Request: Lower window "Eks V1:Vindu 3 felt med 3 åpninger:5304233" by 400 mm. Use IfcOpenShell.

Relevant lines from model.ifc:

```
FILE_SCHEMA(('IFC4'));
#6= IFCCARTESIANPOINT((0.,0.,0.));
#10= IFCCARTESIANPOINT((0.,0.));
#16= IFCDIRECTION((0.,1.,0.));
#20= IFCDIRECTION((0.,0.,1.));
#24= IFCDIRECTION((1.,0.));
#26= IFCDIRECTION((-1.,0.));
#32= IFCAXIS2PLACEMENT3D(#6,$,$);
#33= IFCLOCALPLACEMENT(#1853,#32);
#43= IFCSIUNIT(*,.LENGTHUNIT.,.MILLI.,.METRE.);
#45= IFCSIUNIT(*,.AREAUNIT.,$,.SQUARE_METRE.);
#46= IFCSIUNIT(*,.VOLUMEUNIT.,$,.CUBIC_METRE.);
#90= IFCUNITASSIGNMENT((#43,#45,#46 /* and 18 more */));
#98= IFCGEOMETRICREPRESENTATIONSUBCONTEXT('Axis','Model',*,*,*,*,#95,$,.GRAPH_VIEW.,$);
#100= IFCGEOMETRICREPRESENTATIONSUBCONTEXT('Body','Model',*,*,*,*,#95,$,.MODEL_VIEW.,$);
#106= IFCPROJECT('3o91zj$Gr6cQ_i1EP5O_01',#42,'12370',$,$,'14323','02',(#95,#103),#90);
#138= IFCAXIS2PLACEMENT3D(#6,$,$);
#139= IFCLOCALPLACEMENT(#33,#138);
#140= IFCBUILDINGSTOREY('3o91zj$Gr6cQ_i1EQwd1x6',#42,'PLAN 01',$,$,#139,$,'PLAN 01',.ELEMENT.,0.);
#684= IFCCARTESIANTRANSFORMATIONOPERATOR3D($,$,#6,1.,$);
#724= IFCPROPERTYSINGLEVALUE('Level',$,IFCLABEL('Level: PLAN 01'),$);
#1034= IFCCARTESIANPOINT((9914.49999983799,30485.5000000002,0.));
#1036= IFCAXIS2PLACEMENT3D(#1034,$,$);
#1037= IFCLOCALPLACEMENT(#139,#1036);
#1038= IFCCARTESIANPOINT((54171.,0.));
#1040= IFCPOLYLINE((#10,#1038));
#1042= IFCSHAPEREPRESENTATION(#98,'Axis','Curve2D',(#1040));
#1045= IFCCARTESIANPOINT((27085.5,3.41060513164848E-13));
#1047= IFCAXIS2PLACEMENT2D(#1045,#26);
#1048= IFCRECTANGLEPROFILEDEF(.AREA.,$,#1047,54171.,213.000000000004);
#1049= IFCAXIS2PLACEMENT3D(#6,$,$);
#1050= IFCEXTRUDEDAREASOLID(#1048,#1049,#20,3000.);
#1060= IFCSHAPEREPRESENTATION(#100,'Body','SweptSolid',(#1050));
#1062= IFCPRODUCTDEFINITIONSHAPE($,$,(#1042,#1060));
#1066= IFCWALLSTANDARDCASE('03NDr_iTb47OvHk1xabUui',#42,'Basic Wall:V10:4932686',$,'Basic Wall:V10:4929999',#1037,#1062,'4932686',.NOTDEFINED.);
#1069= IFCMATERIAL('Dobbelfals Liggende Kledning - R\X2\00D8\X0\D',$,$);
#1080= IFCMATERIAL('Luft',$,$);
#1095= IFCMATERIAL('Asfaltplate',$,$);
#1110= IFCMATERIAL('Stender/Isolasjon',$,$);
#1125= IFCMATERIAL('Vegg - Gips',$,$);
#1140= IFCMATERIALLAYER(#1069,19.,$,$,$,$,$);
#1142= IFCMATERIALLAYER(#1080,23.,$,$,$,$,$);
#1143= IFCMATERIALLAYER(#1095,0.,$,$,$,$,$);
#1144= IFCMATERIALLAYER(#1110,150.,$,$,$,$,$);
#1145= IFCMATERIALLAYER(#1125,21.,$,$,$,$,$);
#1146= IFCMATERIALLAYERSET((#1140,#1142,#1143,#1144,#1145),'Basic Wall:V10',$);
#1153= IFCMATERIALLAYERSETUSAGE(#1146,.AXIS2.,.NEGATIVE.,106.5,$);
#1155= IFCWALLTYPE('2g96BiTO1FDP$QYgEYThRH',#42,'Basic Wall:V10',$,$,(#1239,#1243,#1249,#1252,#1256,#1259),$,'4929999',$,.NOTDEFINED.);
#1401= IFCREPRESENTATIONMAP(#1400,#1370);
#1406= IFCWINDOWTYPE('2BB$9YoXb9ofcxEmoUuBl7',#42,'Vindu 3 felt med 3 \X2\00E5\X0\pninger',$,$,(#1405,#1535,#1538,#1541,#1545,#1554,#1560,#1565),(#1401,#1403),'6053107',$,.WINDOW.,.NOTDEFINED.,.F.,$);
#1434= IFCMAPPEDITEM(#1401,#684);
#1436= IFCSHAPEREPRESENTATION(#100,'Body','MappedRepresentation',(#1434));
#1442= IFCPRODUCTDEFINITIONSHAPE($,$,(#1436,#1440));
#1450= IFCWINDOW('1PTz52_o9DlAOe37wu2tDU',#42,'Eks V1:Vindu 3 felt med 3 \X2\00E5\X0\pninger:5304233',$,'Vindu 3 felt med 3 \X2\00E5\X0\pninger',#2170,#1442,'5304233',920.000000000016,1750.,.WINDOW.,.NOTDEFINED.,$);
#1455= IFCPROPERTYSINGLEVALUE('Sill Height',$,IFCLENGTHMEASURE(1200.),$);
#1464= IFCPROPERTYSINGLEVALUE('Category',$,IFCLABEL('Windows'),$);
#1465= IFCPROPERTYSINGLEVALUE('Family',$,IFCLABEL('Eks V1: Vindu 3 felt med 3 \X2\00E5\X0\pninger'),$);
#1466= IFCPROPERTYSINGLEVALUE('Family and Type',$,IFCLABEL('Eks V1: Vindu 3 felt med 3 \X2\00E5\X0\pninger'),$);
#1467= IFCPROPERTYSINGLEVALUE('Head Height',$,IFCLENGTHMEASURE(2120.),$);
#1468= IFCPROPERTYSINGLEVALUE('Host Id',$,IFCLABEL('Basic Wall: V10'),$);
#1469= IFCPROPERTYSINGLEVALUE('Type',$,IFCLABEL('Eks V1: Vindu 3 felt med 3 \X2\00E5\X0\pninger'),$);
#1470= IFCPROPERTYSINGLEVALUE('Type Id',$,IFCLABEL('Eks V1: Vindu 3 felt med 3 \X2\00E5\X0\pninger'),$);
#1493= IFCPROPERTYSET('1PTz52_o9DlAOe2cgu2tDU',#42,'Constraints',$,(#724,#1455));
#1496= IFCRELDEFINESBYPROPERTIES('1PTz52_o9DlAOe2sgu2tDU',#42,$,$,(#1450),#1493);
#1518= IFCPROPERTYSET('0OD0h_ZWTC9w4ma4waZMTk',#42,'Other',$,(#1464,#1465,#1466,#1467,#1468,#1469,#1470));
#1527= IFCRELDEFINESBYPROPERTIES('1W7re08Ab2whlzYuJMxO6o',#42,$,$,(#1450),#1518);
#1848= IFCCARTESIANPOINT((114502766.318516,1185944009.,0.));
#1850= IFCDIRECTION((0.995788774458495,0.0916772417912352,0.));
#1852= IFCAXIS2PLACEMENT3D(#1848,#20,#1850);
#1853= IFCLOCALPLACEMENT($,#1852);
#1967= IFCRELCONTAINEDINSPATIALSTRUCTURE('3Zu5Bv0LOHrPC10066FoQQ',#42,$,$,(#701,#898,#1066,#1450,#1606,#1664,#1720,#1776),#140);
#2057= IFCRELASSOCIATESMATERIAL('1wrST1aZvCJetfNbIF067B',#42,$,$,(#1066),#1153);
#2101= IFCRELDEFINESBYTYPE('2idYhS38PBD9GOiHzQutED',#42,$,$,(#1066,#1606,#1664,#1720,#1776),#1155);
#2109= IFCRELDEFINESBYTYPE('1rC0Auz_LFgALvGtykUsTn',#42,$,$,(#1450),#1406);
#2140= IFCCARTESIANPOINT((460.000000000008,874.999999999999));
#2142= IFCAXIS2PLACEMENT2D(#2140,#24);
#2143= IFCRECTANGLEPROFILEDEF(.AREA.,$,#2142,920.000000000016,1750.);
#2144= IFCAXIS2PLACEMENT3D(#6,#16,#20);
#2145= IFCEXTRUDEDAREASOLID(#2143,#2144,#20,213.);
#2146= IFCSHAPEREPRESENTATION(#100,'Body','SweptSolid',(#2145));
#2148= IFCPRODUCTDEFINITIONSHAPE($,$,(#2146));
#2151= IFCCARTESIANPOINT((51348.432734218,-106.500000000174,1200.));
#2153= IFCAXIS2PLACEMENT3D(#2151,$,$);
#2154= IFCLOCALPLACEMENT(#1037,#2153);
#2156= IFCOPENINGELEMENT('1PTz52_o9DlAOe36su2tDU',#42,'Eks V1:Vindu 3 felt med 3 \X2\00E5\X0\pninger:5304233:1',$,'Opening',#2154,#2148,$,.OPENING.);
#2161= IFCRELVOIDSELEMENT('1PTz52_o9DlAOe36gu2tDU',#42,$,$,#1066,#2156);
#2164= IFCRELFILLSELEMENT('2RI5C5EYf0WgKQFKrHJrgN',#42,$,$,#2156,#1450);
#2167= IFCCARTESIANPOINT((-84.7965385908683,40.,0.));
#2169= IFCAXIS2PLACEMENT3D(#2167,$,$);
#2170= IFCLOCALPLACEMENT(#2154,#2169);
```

```python
import numpy as np
import ifcopenshell
import ifcopenshell.api.geometry
import ifcopenshell.api.pset
import ifcopenshell.util.element
import ifcopenshell.util.placement
import ifcopenshell.util.unit

model = ifcopenshell.open("model.ifc")
unit_scale = ifcopenshell.util.unit.calculate_unit_scale(model)

window = model.by_guid("1PTz52_o9DlAOe37wu2tDU")
opening = window.FillsVoids[0].RelatingOpeningElement
dz = -0.4 / unit_scale

shift = np.array([0.0, 0.0, dz])
# The window is placed relative to its opening, so it follows when the opening moves.
matrix = ifcopenshell.util.placement.get_local_placement(opening.ObjectPlacement)
matrix[:3, 3] += shift
ifcopenshell.api.geometry.edit_object_placement(
    model, product=opening, matrix=matrix, is_si=False, should_transform_children=True
)

# Keep the stored heights in step.
pset = model.by_id(ifcopenshell.util.element.get_pset(window, "Constraints", should_inherit=False)["id"])
ifcopenshell.api.pset.edit_pset(model, pset=pset, properties={
    "Sill Height": model.create_entity("IfcLengthMeasure", ifcopenshell.util.element.get_pset(window, "Constraints", "Sill Height") + dz),
})
pset = model.by_id(ifcopenshell.util.element.get_pset(window, "Other", should_inherit=False)["id"])
ifcopenshell.api.pset.edit_pset(model, pset=pset, properties={
    "Head Height": model.create_entity("IfcLengthMeasure", ifcopenshell.util.element.get_pset(window, "Other", "Head Height") + dz),
})

print(f"moved by {dz * unit_scale:+.3f} m")

model.write("model-out.ifc")
```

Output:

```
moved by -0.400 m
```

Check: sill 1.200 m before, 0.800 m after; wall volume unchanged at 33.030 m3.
